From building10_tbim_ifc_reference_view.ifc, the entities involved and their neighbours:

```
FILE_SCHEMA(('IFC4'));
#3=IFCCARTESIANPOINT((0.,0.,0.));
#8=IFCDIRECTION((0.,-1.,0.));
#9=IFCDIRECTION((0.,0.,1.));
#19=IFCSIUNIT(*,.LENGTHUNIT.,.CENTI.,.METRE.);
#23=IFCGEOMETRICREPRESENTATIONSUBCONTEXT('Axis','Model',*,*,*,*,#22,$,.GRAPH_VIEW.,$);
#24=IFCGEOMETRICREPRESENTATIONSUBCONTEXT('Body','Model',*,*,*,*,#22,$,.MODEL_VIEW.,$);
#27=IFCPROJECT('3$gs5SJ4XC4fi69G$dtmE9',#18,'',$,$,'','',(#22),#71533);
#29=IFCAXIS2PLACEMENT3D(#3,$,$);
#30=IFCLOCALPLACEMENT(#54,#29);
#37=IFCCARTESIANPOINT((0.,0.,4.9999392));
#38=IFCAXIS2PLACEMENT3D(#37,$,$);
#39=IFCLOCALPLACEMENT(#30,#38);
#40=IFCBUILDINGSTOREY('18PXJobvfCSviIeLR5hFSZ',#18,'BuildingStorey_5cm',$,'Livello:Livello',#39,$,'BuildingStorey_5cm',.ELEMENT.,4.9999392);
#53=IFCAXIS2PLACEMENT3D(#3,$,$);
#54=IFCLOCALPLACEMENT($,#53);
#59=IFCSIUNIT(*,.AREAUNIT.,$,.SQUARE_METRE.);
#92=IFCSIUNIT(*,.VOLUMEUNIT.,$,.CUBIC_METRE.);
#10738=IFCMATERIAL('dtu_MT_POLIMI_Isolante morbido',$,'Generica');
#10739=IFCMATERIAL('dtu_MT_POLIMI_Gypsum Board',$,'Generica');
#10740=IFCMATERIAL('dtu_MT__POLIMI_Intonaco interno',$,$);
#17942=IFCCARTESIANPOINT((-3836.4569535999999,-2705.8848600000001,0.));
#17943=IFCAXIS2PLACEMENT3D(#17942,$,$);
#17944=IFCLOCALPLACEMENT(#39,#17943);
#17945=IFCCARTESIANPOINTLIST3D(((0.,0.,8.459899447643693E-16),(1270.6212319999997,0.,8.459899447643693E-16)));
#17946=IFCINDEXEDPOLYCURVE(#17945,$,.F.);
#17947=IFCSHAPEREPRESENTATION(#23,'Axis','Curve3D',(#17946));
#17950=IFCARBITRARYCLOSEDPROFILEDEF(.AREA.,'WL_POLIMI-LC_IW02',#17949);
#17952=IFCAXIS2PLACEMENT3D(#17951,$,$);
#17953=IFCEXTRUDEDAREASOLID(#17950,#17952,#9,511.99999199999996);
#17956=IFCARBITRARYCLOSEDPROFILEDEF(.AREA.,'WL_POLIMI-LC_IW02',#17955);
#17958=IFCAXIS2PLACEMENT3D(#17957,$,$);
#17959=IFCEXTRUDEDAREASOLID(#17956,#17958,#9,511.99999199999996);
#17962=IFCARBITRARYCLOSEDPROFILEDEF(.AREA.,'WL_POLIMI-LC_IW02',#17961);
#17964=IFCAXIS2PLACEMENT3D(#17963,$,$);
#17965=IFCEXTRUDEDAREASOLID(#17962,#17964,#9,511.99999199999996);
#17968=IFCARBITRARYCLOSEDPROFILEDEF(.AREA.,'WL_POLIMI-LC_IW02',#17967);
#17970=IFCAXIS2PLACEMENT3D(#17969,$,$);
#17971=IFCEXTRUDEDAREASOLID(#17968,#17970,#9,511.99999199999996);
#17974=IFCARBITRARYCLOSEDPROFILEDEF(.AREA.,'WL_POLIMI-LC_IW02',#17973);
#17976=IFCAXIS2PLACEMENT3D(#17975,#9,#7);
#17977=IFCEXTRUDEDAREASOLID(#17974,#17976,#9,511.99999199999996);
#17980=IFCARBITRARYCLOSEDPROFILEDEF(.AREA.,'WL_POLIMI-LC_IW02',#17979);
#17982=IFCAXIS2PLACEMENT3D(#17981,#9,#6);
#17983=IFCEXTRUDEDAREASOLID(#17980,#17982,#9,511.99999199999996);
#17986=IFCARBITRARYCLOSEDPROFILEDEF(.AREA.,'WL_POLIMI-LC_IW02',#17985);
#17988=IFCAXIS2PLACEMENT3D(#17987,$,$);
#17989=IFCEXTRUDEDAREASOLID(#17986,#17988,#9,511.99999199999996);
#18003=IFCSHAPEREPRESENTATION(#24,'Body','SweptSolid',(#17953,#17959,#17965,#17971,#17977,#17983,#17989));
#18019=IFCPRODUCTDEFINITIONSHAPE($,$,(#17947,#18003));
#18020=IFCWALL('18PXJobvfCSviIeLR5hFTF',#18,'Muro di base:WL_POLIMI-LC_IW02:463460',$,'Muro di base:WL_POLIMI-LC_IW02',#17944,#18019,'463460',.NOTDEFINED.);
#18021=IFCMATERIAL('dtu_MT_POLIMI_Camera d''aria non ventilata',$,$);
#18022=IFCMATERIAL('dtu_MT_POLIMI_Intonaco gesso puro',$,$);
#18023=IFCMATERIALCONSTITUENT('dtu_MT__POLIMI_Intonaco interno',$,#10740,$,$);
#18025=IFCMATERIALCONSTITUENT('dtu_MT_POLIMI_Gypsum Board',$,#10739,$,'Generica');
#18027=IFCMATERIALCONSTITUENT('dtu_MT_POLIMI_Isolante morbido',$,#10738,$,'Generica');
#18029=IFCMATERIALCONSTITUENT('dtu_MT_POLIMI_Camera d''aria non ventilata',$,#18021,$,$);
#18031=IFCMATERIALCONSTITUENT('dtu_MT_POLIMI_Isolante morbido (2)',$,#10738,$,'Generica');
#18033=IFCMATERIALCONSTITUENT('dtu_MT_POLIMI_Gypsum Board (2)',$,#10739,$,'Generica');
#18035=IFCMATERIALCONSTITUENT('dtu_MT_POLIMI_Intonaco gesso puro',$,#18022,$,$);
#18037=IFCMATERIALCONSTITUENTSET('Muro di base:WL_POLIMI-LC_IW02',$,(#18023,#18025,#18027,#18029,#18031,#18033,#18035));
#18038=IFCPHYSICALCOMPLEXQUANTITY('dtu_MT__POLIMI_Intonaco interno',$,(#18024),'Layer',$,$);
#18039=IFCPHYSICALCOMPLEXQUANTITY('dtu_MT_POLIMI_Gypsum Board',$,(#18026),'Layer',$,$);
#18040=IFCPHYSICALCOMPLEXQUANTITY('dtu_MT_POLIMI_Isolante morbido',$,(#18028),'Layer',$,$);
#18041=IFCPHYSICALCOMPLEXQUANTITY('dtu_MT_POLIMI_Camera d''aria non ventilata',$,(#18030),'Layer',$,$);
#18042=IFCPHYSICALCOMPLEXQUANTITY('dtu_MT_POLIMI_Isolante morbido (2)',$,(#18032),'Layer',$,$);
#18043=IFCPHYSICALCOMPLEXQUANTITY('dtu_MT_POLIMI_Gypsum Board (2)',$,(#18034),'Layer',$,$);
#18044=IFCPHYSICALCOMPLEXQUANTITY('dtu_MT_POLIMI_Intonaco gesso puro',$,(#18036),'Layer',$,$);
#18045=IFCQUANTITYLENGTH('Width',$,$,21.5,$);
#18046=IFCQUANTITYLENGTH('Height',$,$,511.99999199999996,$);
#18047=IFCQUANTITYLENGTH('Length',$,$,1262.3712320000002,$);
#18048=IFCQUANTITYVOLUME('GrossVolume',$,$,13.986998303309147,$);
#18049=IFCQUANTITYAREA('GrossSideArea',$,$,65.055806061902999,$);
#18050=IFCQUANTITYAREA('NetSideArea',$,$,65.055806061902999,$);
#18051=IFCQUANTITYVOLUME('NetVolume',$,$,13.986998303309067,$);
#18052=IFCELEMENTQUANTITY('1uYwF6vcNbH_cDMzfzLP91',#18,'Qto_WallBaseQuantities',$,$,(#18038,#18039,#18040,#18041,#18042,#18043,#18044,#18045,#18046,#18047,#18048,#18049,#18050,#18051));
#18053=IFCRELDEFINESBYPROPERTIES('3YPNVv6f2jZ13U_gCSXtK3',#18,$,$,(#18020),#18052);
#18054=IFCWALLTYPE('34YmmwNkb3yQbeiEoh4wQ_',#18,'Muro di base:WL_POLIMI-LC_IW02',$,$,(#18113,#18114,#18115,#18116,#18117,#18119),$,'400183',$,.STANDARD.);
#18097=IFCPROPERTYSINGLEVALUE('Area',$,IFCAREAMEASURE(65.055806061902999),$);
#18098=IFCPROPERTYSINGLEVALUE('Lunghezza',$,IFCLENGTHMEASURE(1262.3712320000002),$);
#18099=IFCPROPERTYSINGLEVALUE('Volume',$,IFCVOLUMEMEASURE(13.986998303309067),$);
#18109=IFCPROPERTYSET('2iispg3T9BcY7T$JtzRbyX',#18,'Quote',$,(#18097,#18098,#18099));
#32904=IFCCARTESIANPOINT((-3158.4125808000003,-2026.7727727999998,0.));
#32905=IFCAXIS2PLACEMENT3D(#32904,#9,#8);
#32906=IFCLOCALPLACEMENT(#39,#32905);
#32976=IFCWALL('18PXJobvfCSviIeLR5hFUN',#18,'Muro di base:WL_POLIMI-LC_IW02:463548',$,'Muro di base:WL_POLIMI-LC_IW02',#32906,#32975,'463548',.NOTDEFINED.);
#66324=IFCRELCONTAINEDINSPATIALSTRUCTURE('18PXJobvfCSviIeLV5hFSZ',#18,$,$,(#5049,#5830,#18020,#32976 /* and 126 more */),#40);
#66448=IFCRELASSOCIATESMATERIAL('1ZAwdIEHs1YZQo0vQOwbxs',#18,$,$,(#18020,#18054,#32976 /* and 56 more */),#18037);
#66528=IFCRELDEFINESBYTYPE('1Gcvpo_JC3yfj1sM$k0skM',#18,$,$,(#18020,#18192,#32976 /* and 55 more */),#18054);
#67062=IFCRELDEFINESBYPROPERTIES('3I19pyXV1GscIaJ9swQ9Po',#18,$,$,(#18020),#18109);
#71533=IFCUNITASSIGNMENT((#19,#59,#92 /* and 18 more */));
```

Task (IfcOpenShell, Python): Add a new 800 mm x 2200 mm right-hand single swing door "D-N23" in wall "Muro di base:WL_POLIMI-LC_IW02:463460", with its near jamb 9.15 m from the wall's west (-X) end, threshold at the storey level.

```python
import numpy as np
import ifcopenshell
import ifcopenshell.api.feature
import ifcopenshell.api.geometry
import ifcopenshell.api.pset
import ifcopenshell.api.root
import ifcopenshell.api.spatial
import ifcopenshell.geom
import ifcopenshell.util.element
import ifcopenshell.util.placement
import ifcopenshell.util.representation
import ifcopenshell.util.shape
import ifcopenshell.util.unit

model = ifcopenshell.open("building10_tbim_ifc_reference_view.ifc")
unit_scale = ifcopenshell.util.unit.calculate_unit_scale(model)
area_scale = ifcopenshell.util.unit.calculate_unit_scale(model, "AREAUNIT")
volume_scale = ifcopenshell.util.unit.calculate_unit_scale(model, "VOLUMEUNIT")
settings = ifcopenshell.geom.settings()


def volume(element):
    """Net volume in cubic metres, openings subtracted."""
    shape = ifcopenshell.geom.create_shape(settings, element)
    return ifcopenshell.util.shape.get_volume(shape.geometry)


wall = model.by_guid("18PXJobvfCSviIeLR5hFTF")
storey = ifcopenshell.util.element.get_container(wall, ifc_class="IfcBuildingStorey")
context = ifcopenshell.util.representation.get_context(model, "Model", "Body", "MODEL_VIEW")
before = volume(wall)

width, height, from_end, sill = 0.8, 2.2, 9.15, 0.0  # metres

# The wall runs along its own X axis, and the end named is its -X end.
wall_shape = ifcopenshell.geom.create_shape(settings, wall)
x, y, z = ifcopenshell.util.shape.get_vertices(wall_shape.geometry).T
start = x.min() + from_end
face, thickness = float(y.min()), float(y.max() - y.min())
wall_matrix = ifcopenshell.util.placement.get_local_placement(wall.ObjectPlacement)
level = ifcopenshell.util.placement.get_local_placement(storey.ObjectPlacement)[2, 3]


def in_wall(x, y):
    """Placement at x, y metres in the wall's axes, at sill height."""
    matrix = wall_matrix.copy()
    matrix[:, 3] = wall_matrix @ np.array([x / unit_scale, y / unit_scale, 0.0, 1.0])
    matrix[2, 3] = level + sill / unit_scale
    return matrix


# Opening: a box that overshoots both wall faces by 50 mm.
opening = ifcopenshell.api.root.create_entity(model, ifc_class="IfcOpeningElement", predefined_type="OPENING")
box = ifcopenshell.api.geometry.add_wall_representation(
    model, context=context, length=width, height=height, thickness=thickness + 0.1
)
ifcopenshell.api.geometry.assign_representation(model, product=opening, representation=box)
ifcopenshell.api.geometry.edit_object_placement(model, product=opening, matrix=in_wall(start, face - 0.05), is_si=False)
ifcopenshell.api.feature.add_feature(model, feature=opening, element=wall)

door = ifcopenshell.api.root.create_entity(model, ifc_class="IfcDoor", name="D-N23", predefined_type="DOOR")
door.OverallWidth, door.OverallHeight = width / unit_scale, height / unit_scale
door.OperationType = "SINGLE_SWING_RIGHT"
body = ifcopenshell.api.geometry.add_door_representation(
    model,
    context=context,
    overall_width=door.OverallWidth,
    overall_height=door.OverallHeight,
    operation_type="SINGLE_SWING_RIGHT",
    lining_properties={"LiningDepth": thickness / unit_scale, "ThresholdDepth": thickness / unit_scale},
)
ifcopenshell.api.geometry.assign_representation(model, product=door, representation=body)
ifcopenshell.api.spatial.assign_container(model, products=[door], relating_structure=storey)
ifcopenshell.api.feature.add_filling(model, opening=opening, element=door)

# The lining spans the wall, so the door starts at the wall face.
ifcopenshell.api.geometry.edit_object_placement(model, product=door, matrix=in_wall(start, face), is_si=False)

after = volume(wall)

# Update the wall's stored quantities.
qto = model.by_id(ifcopenshell.util.element.get_pset(wall, "Qto_WallBaseQuantities", should_inherit=False)["id"])
ifcopenshell.api.pset.edit_qto(model, qto=qto, properties={
    "NetSideArea": after / thickness / area_scale,
    "NetVolume": after / volume_scale,
})
pset = model.by_id(ifcopenshell.util.element.get_pset(wall, "Quote", should_inherit=False)["id"])
ifcopenshell.api.pset.edit_pset(model, pset=pset, properties={
    "Area": model.create_entity("IfcAreaMeasure", after / thickness / area_scale),
    "Volume": model.create_entity("IfcVolumeMeasure", after / volume_scale),
})

print(f"wall volume {before:.3f} -> {after:.3f} m3")

model.write("building10_tbim_ifc_reference_view_edited.ifc")
```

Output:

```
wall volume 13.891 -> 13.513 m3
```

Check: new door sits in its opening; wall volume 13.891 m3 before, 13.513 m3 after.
